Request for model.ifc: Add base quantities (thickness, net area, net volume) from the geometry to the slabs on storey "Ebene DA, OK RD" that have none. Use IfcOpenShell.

First a look at what the model holds.

```python
import ifcopenshell
import ifcopenshell.util.element
import ifcopenshell.util.unit

model = ifcopenshell.open("model.ifc")
print(model.schema)
for unit_type in ("LENGTHUNIT", "AREAUNIT", "VOLUMEUNIT"):
    print(unit_type, ifcopenshell.util.unit.calculate_unit_scale(model, unit_type))
storey = next(s for s in model.by_type("IfcBuildingStorey") if s.Name == "Ebene DA, OK RD")
slabs = [e for e in ifcopenshell.util.element.get_decomposition(storey) if e.is_a("IfcSlab")]
for e in sorted(slabs, key=lambda e: e.id()):
    print(e.id(), e.is_a(), e.Name, list(ifcopenshell.util.element.get_psets(e, qtos_only=True)), sep=" | ")
```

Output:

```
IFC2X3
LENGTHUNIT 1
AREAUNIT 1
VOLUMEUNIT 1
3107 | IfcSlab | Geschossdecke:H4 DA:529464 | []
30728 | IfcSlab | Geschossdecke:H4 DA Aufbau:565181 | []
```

```python
import ifcopenshell
import ifcopenshell.api.pset
import ifcopenshell.geom
import ifcopenshell.util.element
import ifcopenshell.util.shape
import ifcopenshell.util.unit

model = ifcopenshell.open("model.ifc")
unit_scale = ifcopenshell.util.unit.calculate_unit_scale(model)
area_scale = ifcopenshell.util.unit.calculate_unit_scale(model, "AREAUNIT")
volume_scale = ifcopenshell.util.unit.calculate_unit_scale(model, "VOLUMEUNIT")
settings = ifcopenshell.geom.settings()

storey = next(s for s in model.by_type("IfcBuildingStorey") if s.Name == "Ebene DA, OK RD")
slabs = [e for e in ifcopenshell.util.element.get_decomposition(storey) if e.is_a("IfcSlab")]

for e in sorted(slabs, key=lambda e: e.id()):
    if ifcopenshell.util.element.get_psets(e, qtos_only=True, should_inherit=False):
        continue
    # Geometry comes back in metres, in the element's own axes.
    shape = ifcopenshell.geom.create_shape(settings, e)
    values = {
        "Width": ifcopenshell.util.shape.get_z(shape.geometry) / unit_scale,
        "NetArea": ifcopenshell.util.shape.get_footprint_area(shape.geometry) / area_scale,
        "NetVolume": ifcopenshell.util.shape.get_volume(shape.geometry) / volume_scale,
    }
    qto = ifcopenshell.api.pset.add_qto(model, product=e, name="BaseQuantities")
    ifcopenshell.api.pset.edit_qto(model, qto=qto, properties=values)
    print(e.id(), {k: round(v, 3) for k, v in values.items()})

model.write("model_edited.ifc")
```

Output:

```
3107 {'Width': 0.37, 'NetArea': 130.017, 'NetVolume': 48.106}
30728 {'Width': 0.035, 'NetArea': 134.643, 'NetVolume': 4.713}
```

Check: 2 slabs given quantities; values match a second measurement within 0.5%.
